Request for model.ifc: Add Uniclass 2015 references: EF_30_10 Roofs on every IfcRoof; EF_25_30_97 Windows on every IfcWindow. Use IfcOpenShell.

First a look at what the model holds.

```python
import ifcopenshell

model = ifcopenshell.open("model.ifc")
print(model.schema)
print("classifications:", [c.Name for c in model.by_type("IfcClassification")])
for ifc_class in ("IfcDoor", "IfcRoof", "IfcStair", "IfcWall", "IfcWindow"):
    print(ifc_class, len(model.by_type(ifc_class)))
```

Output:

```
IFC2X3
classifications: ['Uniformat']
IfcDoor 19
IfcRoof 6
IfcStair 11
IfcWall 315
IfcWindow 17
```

```python
import ifcopenshell
import ifcopenshell.api.classification

model = ifcopenshell.open("model.ifc")

# IFC2X3 requires Source and Edition and has no link from the project to the system.
system = model.create_entity("IfcClassification", Source="NBS", Edition="2015", Name="Uniclass 2015")

codes = {
    "IfcRoof": ("EF_30_10", "Roofs"),
    "IfcWindow": ("EF_25_30_97", "Windows"),
}
for ifc_class, (code, name) in codes.items():
    products = model.by_type(ifc_class)
    ifcopenshell.api.classification.add_reference(
        model, products=products, classification=system, identification=code, name=name
    )
    print(code, len(products))

model.write("model_v2.ifc")
```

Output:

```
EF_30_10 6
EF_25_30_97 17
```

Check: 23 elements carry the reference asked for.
